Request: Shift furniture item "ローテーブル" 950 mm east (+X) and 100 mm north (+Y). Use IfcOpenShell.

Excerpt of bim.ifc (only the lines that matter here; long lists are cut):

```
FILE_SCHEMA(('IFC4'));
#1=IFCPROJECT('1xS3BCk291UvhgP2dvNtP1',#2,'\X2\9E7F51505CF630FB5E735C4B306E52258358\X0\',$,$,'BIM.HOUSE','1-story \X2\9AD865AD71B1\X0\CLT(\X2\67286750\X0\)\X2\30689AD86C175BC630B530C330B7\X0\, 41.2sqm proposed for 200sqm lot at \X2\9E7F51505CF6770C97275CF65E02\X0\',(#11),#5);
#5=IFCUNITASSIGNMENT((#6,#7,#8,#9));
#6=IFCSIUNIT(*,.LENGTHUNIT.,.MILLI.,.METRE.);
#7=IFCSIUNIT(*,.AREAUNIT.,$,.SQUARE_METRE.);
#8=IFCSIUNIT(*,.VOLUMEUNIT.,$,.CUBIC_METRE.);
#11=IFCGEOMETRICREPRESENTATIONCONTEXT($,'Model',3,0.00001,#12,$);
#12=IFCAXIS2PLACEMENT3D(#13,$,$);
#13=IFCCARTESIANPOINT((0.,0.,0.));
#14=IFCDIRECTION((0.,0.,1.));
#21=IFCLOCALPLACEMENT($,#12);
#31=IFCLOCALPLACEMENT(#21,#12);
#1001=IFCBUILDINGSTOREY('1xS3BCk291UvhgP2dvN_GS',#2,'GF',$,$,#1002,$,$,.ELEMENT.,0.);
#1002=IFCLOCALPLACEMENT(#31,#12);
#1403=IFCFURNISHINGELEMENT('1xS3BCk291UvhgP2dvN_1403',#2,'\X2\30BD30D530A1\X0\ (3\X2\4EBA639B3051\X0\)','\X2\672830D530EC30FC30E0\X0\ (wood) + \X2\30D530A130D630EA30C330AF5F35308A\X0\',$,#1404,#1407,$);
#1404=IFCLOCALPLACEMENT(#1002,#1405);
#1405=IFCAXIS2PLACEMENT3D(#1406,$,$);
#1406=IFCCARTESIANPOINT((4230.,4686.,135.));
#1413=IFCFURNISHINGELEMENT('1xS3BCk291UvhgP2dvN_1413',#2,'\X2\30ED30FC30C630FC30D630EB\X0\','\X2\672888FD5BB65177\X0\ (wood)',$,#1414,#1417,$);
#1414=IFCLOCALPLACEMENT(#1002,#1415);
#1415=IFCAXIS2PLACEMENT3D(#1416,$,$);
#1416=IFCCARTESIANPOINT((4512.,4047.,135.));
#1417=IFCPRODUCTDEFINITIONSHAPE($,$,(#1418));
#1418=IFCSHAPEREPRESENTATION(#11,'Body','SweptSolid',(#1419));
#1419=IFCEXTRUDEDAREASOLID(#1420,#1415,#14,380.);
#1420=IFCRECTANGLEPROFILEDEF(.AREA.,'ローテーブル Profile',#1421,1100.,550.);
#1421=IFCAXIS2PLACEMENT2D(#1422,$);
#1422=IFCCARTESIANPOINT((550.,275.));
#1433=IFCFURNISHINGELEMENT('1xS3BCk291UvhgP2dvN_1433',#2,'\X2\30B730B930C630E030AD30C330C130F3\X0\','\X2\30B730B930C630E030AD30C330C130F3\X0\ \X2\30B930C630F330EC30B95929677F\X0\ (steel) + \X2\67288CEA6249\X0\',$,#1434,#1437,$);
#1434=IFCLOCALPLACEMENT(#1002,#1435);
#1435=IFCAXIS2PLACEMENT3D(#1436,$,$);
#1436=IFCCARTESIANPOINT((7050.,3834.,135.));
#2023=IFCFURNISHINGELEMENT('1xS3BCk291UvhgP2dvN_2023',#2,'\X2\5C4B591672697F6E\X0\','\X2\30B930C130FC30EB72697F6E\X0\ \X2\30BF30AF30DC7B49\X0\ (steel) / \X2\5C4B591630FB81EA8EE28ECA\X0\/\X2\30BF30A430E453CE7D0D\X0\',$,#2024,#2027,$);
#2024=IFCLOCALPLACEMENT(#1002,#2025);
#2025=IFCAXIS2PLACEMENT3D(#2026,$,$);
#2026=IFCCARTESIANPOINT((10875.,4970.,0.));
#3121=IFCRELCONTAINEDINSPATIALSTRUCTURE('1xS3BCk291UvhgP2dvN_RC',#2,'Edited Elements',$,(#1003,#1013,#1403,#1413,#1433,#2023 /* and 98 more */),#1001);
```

```python
import ifcopenshell
import ifcopenshell.api.geometry
import ifcopenshell.util.placement

model = ifcopenshell.open("bim.ifc")

item = model.by_guid("1xS3BCk291UvhgP2dvN_1413")
matrix = ifcopenshell.util.placement.get_local_placement(item.ObjectPlacement)
matrix[0, 3] += 950.0
matrix[1, 3] += 100.0
ifcopenshell.api.geometry.edit_object_placement(model, product=item, matrix=matrix, is_si=False)

print(ifcopenshell.util.placement.get_local_placement(item.ObjectPlacement).round(3) + 0.0)

model.write("bim_edited.ifc")
```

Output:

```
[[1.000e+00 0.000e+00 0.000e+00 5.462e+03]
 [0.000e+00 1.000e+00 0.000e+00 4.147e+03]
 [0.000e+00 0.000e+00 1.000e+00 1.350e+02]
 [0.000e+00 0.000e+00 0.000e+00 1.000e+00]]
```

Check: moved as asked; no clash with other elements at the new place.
